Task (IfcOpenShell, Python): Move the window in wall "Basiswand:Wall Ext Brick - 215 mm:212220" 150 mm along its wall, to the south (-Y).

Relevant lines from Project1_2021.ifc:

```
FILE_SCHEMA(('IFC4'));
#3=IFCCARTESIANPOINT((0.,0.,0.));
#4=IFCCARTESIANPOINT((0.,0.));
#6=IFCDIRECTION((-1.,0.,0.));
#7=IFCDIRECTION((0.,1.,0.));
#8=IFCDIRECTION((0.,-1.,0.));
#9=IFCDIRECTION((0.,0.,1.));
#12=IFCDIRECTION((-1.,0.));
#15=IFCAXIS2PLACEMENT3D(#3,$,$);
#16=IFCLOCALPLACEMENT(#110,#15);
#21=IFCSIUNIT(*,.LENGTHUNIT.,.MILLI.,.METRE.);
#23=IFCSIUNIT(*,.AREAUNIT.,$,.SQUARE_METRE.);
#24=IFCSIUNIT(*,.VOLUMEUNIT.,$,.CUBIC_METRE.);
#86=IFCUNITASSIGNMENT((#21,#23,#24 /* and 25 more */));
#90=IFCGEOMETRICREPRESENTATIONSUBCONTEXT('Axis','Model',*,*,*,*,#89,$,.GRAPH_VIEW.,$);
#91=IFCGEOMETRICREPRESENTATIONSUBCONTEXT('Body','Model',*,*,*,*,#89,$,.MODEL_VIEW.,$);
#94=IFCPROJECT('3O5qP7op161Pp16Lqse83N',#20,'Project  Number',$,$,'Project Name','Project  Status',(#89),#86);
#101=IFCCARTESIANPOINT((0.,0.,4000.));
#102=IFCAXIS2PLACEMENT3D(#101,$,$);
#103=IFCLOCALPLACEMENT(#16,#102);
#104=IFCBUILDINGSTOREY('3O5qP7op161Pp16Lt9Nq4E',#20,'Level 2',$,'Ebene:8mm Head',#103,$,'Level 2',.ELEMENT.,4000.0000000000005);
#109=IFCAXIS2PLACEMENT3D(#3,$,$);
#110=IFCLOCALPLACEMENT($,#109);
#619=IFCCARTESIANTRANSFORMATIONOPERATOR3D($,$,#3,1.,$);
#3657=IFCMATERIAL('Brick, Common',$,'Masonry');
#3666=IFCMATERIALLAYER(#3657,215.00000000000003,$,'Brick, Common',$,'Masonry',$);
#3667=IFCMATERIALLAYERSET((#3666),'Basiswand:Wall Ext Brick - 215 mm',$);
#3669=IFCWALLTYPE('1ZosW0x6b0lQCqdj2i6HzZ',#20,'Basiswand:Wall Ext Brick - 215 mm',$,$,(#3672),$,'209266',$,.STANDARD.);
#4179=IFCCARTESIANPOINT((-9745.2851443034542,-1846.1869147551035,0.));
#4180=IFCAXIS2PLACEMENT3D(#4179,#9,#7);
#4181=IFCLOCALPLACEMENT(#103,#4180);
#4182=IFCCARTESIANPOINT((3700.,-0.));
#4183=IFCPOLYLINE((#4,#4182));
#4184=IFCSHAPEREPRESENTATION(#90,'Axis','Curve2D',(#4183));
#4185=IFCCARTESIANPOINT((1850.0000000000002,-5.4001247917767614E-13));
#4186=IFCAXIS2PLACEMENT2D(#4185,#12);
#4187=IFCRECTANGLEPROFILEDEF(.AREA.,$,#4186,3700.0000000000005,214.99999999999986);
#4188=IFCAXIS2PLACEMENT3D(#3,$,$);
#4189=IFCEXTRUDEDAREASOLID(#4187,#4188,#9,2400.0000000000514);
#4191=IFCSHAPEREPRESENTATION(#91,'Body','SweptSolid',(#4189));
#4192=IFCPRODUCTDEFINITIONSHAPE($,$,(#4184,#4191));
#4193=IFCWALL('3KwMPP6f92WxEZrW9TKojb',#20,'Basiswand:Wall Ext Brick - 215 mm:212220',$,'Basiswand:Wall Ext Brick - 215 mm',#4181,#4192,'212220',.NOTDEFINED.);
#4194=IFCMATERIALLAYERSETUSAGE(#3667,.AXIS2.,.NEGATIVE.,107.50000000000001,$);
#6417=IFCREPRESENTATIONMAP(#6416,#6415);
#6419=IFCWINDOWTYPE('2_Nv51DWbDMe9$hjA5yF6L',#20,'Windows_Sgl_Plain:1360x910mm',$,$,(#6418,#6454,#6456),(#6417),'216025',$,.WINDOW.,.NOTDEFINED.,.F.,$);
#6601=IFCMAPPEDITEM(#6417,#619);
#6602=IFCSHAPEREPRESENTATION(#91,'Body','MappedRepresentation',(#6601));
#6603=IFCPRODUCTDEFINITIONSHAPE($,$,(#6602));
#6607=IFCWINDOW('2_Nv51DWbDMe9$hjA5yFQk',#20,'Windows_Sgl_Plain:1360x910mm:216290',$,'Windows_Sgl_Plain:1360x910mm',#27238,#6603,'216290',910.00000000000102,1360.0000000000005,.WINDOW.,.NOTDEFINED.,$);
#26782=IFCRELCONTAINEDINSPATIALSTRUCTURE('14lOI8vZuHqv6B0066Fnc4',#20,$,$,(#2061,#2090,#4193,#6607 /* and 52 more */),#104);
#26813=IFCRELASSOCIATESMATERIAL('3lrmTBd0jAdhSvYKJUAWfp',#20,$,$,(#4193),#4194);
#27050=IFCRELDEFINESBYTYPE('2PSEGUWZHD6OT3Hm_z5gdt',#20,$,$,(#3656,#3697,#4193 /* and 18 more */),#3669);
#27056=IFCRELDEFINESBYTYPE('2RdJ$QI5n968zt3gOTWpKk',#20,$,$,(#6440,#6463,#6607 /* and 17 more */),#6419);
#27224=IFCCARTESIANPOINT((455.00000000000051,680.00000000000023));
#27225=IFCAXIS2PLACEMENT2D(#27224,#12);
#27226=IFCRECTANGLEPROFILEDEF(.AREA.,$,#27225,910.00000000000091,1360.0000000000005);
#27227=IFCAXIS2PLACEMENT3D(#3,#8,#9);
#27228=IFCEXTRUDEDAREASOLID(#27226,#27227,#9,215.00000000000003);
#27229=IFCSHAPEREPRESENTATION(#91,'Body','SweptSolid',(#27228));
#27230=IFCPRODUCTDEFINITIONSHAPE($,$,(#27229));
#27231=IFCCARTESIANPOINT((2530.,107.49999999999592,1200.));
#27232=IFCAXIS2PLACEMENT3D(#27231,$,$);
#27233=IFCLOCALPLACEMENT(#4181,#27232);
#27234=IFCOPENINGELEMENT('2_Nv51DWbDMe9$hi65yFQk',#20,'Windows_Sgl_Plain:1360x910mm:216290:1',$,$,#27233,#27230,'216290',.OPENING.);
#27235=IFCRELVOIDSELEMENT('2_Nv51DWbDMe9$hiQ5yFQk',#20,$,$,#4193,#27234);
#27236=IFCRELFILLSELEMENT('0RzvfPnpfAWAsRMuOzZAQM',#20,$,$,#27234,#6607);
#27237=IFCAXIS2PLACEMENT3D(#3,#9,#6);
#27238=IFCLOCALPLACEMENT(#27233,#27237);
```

```python
import ifcopenshell
import ifcopenshell.api.geometry
import ifcopenshell.util.placement
import ifcopenshell.util.unit

model = ifcopenshell.open("Project1_2021.ifc")
unit_scale = ifcopenshell.util.unit.calculate_unit_scale(model)

window = model.by_id(6607)
opening = window.FillsVoids[0].RelatingOpeningElement
wall = opening.VoidsElements[0].RelatingBuildingElement

wall_matrix = ifcopenshell.util.placement.get_local_placement(wall.ObjectPlacement)
shift = wall_matrix[:3, 0] * -0.15 / unit_scale
before = ifcopenshell.util.placement.get_local_placement(window.ObjectPlacement)[:3, 3].copy()

# The window is placed relative to its opening, so it follows when the opening moves.
matrix = ifcopenshell.util.placement.get_local_placement(opening.ObjectPlacement)
matrix[:3, 3] += shift
ifcopenshell.api.geometry.edit_object_placement(
    model, product=opening, matrix=matrix, is_si=False, should_transform_children=True
)

after = ifcopenshell.util.placement.get_local_placement(window.ObjectPlacement)[:3, 3]
print("window moved by", (after - before).round(3) + 0.0)

model.write("Project1_2021_rev.ifc")
```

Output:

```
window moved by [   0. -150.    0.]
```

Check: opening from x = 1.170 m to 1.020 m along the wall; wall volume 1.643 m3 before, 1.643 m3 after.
